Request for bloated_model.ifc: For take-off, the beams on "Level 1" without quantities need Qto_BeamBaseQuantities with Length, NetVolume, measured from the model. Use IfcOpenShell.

First a look at what the model holds.

```python
import ifcopenshell
import ifcopenshell.util.element
import ifcopenshell.util.unit

model = ifcopenshell.open("bloated_model.ifc")
print(model.schema)
for unit_type in ("LENGTHUNIT", "AREAUNIT", "VOLUMEUNIT"):
    print(unit_type, ifcopenshell.util.unit.calculate_unit_scale(model, unit_type))
storey = next(s for s in model.by_type("IfcBuildingStorey") if s.Name == "Level 1")
beams = [e for e in ifcopenshell.util.element.get_decomposition(storey) if e.is_a("IfcBeam")]
for e in sorted(beams, key=lambda e: e.id()):
    print(e.id(), e.is_a(), e.Name, list(ifcopenshell.util.element.get_psets(e, qtos_only=True)), sep=" | ")
```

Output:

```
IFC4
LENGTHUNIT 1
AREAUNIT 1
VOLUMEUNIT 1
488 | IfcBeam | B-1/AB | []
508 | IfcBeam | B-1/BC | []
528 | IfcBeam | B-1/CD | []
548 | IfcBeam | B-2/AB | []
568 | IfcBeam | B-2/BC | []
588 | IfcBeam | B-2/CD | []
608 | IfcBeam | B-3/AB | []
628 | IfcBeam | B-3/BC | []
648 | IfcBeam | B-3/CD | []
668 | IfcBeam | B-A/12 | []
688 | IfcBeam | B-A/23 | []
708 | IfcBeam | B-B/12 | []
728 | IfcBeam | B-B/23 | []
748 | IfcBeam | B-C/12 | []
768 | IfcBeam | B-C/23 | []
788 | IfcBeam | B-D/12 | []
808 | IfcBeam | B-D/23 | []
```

```python
import ifcopenshell
import ifcopenshell.api.pset
import ifcopenshell.geom
import ifcopenshell.util.element
import ifcopenshell.util.shape
import ifcopenshell.util.unit

model = ifcopenshell.open("bloated_model.ifc")
unit_scale = ifcopenshell.util.unit.calculate_unit_scale(model)
volume_scale = ifcopenshell.util.unit.calculate_unit_scale(model, "VOLUMEUNIT")
settings = ifcopenshell.geom.settings()

storey = next(s for s in model.by_type("IfcBuildingStorey") if s.Name == "Level 1")
beams = [e for e in ifcopenshell.util.element.get_decomposition(storey) if e.is_a("IfcBeam")]

for e in sorted(beams, key=lambda e: e.id()):
    if ifcopenshell.util.element.get_psets(e, qtos_only=True, should_inherit=False):
        continue
    # Geometry comes back in metres, in the element's own axes.
    shape = ifcopenshell.geom.create_shape(settings, e)
    values = {
        "Length": ifcopenshell.util.shape.get_max_xyz(shape.geometry) / unit_scale,
        "NetVolume": ifcopenshell.util.shape.get_volume(shape.geometry) / volume_scale,
    }
    qto = ifcopenshell.api.pset.add_qto(model, product=e, name="Qto_BeamBaseQuantities")
    ifcopenshell.api.pset.edit_qto(model, qto=qto, properties=values)
    print(e.id(), {k: round(v, 3) for k, v in values.items()})

model.write("bloated_model_edited.ifc")
```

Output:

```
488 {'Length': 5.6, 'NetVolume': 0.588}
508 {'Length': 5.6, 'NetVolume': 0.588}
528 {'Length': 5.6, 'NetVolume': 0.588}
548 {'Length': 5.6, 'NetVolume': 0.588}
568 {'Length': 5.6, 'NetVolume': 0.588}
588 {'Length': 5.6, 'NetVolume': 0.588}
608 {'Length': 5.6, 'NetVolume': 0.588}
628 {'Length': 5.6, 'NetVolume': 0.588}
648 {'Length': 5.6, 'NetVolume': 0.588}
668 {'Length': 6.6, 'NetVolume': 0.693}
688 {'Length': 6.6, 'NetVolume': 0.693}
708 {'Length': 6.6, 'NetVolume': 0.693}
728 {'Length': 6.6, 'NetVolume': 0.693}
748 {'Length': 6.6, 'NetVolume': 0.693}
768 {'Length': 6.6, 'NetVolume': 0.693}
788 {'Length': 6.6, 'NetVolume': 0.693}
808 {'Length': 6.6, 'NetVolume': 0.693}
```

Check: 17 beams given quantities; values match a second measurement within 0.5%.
